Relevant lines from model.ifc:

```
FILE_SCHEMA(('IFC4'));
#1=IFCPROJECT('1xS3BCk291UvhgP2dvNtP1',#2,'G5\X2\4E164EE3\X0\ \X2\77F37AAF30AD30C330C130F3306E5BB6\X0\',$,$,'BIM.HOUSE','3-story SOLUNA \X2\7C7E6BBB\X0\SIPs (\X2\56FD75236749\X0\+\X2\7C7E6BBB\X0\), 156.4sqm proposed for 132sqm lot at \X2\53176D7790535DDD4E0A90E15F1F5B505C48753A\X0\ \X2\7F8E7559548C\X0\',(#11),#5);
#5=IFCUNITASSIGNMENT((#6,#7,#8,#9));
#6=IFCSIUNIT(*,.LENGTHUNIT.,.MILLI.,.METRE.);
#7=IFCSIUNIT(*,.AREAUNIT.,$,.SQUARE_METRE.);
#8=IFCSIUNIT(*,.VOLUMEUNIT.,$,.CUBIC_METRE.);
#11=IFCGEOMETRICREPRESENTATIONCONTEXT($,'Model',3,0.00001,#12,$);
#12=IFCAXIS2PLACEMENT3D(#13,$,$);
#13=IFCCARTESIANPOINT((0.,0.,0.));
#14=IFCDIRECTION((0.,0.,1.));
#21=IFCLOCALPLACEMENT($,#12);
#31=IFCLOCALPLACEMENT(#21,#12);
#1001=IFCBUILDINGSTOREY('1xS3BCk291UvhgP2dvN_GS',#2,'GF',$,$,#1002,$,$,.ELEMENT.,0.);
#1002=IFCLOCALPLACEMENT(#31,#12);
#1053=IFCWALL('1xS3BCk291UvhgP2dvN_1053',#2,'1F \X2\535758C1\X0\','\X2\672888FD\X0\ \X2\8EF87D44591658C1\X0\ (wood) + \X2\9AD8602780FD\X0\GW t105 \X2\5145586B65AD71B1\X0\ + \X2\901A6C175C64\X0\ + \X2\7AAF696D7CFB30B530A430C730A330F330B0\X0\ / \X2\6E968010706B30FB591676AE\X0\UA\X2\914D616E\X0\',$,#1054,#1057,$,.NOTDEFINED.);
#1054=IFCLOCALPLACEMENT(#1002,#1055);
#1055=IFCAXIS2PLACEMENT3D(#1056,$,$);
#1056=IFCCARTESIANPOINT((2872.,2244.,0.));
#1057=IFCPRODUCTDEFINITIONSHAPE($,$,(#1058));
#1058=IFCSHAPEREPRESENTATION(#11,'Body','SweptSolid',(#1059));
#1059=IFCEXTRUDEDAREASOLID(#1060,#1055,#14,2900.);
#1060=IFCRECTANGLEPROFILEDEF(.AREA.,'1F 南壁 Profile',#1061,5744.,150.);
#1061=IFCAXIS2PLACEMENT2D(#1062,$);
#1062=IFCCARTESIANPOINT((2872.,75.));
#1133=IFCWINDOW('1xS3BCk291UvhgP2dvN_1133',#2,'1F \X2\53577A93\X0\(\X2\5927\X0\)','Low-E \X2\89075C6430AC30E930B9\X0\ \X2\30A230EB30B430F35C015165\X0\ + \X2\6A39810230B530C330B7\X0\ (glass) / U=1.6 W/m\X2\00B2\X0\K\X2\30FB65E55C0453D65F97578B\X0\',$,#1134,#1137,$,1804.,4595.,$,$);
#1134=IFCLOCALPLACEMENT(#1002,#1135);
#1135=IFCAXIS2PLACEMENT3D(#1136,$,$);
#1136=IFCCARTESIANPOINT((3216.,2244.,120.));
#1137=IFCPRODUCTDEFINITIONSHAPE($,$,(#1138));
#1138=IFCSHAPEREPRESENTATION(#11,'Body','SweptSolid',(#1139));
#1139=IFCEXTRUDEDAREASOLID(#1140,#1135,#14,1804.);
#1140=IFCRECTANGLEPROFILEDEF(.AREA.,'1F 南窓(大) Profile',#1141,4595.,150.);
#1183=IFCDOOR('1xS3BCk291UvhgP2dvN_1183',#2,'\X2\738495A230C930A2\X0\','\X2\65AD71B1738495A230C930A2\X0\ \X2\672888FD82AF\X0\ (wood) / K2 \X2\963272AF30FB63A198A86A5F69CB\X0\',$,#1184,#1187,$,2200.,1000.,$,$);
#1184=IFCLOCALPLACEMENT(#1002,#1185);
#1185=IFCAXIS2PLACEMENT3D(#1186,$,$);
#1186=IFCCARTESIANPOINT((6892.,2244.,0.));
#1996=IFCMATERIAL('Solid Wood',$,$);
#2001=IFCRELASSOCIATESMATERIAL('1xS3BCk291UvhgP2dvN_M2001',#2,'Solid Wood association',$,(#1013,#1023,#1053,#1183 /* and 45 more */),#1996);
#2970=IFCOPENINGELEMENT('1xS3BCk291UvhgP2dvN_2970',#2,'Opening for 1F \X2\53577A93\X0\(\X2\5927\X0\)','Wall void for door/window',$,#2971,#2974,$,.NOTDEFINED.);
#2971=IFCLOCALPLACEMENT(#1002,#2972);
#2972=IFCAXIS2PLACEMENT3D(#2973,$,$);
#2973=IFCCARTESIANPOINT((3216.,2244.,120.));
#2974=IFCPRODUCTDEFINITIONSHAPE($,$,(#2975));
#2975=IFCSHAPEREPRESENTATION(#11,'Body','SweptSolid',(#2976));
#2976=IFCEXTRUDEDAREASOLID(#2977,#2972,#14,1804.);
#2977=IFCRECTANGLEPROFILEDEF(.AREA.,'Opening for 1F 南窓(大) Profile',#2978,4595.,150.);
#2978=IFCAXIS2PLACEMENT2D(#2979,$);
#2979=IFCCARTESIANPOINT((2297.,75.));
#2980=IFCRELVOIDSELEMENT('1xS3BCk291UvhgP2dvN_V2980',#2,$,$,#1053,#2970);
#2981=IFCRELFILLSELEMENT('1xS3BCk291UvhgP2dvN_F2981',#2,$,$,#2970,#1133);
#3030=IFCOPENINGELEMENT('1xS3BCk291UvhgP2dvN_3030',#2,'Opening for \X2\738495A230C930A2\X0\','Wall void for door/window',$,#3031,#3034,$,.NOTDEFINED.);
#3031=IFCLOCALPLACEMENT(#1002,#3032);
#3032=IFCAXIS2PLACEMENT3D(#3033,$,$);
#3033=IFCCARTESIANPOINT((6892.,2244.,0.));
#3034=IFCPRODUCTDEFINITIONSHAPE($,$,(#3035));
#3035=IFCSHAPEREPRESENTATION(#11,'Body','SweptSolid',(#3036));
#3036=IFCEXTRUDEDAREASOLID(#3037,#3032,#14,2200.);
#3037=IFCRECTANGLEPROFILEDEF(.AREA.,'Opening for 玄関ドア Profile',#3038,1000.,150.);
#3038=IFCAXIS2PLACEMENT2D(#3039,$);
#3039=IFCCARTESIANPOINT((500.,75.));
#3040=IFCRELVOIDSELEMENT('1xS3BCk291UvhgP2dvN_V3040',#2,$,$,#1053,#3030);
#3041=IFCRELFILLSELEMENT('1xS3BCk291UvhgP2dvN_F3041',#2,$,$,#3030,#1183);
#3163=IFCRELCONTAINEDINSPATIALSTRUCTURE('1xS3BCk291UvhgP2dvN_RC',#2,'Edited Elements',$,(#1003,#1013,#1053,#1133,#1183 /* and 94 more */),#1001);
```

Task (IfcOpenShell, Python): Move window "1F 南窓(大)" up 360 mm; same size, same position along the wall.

```python
import numpy as np
import ifcopenshell
import ifcopenshell.api.geometry
import ifcopenshell.util.placement
import ifcopenshell.util.unit

model = ifcopenshell.open("model.ifc")
unit_scale = ifcopenshell.util.unit.calculate_unit_scale(model)

window = model.by_guid("1xS3BCk291UvhgP2dvN_1133")
opening = window.FillsVoids[0].RelatingOpeningElement
dz = 360.0

shift = np.array([0.0, 0.0, dz])
# The window is not placed relative to its opening, so move both.
for product in (opening, window):
    matrix = ifcopenshell.util.placement.get_local_placement(product.ObjectPlacement)
    matrix[:3, 3] += shift
    ifcopenshell.api.geometry.edit_object_placement(model, product=product, matrix=matrix, is_si=False)

print(f"moved by {dz * unit_scale:+.3f} m")

model.write("model_updated.ifc")
```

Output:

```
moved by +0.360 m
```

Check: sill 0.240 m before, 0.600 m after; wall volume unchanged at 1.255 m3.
